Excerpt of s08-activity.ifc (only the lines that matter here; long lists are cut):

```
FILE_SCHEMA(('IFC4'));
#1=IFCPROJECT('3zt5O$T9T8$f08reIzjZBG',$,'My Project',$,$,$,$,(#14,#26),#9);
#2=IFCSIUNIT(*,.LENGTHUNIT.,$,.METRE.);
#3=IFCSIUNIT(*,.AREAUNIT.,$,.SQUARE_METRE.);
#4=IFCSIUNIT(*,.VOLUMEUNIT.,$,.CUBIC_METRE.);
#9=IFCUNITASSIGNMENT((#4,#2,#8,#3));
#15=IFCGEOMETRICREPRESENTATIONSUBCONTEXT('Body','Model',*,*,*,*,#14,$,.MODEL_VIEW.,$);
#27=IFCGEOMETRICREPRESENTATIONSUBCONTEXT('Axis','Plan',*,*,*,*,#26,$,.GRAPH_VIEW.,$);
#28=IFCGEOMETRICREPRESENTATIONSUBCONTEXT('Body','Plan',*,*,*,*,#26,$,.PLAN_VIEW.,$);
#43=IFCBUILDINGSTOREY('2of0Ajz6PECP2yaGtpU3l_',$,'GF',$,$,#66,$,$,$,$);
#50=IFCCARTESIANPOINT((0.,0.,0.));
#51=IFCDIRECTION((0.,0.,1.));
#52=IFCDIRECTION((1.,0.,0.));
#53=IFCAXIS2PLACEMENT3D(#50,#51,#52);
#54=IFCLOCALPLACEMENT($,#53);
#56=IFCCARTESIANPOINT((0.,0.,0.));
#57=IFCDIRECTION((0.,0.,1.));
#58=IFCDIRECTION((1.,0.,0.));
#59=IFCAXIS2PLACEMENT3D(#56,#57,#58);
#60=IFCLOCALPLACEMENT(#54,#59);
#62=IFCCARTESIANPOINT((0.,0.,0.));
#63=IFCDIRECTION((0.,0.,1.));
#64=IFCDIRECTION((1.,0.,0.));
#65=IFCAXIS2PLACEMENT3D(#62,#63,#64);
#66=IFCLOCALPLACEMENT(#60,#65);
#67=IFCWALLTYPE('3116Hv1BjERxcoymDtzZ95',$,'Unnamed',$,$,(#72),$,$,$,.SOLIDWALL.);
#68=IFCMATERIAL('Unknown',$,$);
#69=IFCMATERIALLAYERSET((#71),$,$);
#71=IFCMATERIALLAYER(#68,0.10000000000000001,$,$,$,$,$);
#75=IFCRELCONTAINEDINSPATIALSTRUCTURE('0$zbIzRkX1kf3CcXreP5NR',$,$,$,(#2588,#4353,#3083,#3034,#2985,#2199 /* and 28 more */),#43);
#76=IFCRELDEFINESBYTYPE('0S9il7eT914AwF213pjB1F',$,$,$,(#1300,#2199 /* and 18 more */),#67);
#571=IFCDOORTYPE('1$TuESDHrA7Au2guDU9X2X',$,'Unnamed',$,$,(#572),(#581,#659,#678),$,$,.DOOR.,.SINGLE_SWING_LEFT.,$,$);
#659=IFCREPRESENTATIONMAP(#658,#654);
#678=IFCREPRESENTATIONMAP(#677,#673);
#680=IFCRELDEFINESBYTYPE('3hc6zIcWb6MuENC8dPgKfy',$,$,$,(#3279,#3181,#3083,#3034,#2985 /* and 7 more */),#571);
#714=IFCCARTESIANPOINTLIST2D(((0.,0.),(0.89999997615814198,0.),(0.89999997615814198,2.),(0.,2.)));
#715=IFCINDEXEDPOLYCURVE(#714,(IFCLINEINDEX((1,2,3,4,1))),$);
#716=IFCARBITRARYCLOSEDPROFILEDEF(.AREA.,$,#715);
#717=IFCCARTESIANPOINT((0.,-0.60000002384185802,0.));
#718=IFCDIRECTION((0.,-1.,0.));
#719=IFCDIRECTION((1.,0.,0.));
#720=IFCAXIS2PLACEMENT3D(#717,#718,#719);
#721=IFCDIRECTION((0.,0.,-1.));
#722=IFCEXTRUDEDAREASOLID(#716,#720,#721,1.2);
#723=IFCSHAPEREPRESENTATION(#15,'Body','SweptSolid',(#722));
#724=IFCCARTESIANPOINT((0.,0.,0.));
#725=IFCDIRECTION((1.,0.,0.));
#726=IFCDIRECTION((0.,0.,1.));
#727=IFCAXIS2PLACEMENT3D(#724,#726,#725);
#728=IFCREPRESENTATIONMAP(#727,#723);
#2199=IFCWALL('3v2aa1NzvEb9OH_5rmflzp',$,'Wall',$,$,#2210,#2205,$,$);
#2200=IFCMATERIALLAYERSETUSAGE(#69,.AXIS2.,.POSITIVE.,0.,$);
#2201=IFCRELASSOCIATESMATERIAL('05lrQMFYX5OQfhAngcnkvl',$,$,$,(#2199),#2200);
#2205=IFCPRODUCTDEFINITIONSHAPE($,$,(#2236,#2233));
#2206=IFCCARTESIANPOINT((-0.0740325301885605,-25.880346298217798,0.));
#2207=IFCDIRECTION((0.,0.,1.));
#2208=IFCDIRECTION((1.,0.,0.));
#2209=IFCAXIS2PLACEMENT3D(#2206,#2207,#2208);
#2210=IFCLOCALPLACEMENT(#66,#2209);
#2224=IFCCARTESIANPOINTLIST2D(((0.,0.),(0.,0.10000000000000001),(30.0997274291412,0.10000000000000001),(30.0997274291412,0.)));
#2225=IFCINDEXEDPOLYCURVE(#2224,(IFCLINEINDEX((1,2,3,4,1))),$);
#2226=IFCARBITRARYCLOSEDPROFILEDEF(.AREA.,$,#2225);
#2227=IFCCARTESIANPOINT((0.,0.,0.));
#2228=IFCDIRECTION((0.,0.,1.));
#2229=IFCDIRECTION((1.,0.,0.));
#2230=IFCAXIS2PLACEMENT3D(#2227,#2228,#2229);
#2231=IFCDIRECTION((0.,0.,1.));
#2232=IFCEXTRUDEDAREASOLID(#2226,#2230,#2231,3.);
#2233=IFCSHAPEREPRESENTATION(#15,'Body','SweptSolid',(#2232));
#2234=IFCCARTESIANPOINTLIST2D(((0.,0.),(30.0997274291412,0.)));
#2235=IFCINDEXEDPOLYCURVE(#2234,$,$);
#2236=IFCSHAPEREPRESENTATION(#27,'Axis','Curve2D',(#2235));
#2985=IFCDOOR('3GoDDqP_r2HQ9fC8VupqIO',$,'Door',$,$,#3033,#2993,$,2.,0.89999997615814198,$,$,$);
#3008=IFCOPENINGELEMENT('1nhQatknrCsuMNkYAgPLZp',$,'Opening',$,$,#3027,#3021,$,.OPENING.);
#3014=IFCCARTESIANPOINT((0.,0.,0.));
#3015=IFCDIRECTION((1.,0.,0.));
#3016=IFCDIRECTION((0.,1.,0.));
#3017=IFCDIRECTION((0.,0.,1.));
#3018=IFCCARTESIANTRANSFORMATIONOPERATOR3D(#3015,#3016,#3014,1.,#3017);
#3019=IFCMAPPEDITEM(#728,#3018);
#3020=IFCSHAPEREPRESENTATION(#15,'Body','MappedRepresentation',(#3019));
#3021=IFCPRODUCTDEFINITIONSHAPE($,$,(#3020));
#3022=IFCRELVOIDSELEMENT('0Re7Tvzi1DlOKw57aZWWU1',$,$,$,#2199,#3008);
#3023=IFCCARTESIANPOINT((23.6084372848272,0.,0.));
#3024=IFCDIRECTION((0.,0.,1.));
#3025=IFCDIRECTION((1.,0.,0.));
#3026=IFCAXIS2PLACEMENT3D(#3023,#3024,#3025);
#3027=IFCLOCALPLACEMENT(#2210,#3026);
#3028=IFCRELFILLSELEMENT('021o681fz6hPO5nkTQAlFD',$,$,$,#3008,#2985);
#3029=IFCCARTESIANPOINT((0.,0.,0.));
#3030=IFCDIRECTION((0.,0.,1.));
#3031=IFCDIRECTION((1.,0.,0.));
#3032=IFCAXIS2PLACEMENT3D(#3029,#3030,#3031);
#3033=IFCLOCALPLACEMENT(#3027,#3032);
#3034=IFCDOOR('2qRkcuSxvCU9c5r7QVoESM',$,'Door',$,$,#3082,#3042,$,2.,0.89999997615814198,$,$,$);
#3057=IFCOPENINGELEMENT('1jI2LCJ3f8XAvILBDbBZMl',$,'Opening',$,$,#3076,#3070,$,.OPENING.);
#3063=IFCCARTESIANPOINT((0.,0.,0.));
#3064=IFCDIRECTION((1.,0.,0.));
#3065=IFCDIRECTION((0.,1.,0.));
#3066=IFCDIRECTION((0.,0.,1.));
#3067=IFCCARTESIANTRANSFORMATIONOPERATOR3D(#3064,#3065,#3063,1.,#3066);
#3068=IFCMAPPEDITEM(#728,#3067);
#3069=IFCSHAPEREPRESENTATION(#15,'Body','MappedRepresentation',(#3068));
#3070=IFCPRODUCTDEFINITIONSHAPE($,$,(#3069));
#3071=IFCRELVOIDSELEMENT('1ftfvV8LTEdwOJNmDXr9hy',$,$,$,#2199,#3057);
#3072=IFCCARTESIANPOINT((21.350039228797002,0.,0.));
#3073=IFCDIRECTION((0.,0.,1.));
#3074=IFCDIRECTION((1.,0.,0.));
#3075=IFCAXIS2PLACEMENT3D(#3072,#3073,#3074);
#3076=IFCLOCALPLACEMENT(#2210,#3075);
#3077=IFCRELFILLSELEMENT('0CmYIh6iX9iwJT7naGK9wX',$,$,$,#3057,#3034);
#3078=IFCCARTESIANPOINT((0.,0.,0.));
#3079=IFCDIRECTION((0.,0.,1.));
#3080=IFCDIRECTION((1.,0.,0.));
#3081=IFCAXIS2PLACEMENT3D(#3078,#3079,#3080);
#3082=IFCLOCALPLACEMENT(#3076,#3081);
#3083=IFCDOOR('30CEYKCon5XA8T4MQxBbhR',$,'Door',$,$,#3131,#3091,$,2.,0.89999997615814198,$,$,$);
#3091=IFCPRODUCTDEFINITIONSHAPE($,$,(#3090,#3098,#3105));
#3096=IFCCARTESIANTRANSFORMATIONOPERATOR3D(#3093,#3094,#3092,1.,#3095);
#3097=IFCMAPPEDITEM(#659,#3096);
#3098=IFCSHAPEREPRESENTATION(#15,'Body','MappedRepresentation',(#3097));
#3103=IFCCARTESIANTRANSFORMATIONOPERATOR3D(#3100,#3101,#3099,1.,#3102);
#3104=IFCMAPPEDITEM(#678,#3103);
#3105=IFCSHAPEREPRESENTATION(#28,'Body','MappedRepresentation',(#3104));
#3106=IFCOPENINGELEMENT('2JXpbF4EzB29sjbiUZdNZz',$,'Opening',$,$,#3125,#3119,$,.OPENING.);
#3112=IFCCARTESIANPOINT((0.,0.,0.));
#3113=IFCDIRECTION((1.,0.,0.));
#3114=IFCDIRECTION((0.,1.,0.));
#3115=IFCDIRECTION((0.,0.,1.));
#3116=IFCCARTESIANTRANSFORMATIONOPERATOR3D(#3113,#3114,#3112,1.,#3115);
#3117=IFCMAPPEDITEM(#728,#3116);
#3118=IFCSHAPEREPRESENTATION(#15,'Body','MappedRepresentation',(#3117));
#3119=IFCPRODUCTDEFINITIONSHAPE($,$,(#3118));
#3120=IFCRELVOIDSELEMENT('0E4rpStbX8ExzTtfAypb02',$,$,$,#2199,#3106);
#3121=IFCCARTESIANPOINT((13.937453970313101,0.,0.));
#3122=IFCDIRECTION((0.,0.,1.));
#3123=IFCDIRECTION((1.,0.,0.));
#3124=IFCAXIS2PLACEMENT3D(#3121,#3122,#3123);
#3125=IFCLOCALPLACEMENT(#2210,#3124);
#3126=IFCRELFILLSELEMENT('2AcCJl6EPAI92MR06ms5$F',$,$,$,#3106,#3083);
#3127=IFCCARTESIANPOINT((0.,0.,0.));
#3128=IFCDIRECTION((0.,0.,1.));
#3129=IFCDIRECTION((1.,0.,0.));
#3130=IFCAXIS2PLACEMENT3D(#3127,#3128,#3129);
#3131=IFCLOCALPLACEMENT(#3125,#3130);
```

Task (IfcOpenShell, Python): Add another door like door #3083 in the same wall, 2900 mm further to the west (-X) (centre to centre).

```python
import ifcopenshell
import ifcopenshell.api.feature
import ifcopenshell.api.geometry
import ifcopenshell.api.root
import ifcopenshell.geom
import ifcopenshell.util.element
import ifcopenshell.util.placement
import ifcopenshell.util.shape
import ifcopenshell.util.unit

model = ifcopenshell.open("s08-activity.ifc")
unit_scale = ifcopenshell.util.unit.calculate_unit_scale(model)
settings = ifcopenshell.geom.settings()


def volume(element):
    """Net volume in cubic metres, openings subtracted."""
    shape = ifcopenshell.geom.create_shape(settings, element)
    return ifcopenshell.util.shape.get_volume(shape.geometry)


door = model.by_guid("30CEYKCon5XA8T4MQxBbhR")
opening = door.FillsVoids[0].RelatingOpeningElement
wall = opening.VoidsElements[0].RelatingBuildingElement
before = volume(wall)
shift = ifcopenshell.util.placement.get_local_placement(wall.ObjectPlacement)[:3, 0] * -2.9 / unit_scale

# copy_class copies the void relationship, type, container and properties, but no geometry.
new_opening = ifcopenshell.api.root.copy_class(model, product=opening)
new_opening.Representation = ifcopenshell.util.element.copy_deep(
    model, opening.Representation, exclude=["IfcGeometricRepresentationContext", "IfcRepresentationMap"]
)
new_door = ifcopenshell.api.root.copy_class(model, product=door)
new_door.Representation = ifcopenshell.util.element.copy_deep(
    model, door.Representation, exclude=["IfcGeometricRepresentationContext", "IfcRepresentationMap"]
)
ifcopenshell.api.feature.add_filling(model, opening=new_opening, element=new_door)

for old, new in ((opening, new_opening), (door, new_door)):
    matrix = ifcopenshell.util.placement.get_local_placement(old.ObjectPlacement)
    matrix[:3, 3] += shift
    ifcopenshell.api.geometry.edit_object_placement(model, product=new, matrix=matrix, is_si=False)

after = volume(wall)

print(f"wall volume {before:.3f} -> {after:.3f} m3")

model.write("s08-activity_updated.ifc")
```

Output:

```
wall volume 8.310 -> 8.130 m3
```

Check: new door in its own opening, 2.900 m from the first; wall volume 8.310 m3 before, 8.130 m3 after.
